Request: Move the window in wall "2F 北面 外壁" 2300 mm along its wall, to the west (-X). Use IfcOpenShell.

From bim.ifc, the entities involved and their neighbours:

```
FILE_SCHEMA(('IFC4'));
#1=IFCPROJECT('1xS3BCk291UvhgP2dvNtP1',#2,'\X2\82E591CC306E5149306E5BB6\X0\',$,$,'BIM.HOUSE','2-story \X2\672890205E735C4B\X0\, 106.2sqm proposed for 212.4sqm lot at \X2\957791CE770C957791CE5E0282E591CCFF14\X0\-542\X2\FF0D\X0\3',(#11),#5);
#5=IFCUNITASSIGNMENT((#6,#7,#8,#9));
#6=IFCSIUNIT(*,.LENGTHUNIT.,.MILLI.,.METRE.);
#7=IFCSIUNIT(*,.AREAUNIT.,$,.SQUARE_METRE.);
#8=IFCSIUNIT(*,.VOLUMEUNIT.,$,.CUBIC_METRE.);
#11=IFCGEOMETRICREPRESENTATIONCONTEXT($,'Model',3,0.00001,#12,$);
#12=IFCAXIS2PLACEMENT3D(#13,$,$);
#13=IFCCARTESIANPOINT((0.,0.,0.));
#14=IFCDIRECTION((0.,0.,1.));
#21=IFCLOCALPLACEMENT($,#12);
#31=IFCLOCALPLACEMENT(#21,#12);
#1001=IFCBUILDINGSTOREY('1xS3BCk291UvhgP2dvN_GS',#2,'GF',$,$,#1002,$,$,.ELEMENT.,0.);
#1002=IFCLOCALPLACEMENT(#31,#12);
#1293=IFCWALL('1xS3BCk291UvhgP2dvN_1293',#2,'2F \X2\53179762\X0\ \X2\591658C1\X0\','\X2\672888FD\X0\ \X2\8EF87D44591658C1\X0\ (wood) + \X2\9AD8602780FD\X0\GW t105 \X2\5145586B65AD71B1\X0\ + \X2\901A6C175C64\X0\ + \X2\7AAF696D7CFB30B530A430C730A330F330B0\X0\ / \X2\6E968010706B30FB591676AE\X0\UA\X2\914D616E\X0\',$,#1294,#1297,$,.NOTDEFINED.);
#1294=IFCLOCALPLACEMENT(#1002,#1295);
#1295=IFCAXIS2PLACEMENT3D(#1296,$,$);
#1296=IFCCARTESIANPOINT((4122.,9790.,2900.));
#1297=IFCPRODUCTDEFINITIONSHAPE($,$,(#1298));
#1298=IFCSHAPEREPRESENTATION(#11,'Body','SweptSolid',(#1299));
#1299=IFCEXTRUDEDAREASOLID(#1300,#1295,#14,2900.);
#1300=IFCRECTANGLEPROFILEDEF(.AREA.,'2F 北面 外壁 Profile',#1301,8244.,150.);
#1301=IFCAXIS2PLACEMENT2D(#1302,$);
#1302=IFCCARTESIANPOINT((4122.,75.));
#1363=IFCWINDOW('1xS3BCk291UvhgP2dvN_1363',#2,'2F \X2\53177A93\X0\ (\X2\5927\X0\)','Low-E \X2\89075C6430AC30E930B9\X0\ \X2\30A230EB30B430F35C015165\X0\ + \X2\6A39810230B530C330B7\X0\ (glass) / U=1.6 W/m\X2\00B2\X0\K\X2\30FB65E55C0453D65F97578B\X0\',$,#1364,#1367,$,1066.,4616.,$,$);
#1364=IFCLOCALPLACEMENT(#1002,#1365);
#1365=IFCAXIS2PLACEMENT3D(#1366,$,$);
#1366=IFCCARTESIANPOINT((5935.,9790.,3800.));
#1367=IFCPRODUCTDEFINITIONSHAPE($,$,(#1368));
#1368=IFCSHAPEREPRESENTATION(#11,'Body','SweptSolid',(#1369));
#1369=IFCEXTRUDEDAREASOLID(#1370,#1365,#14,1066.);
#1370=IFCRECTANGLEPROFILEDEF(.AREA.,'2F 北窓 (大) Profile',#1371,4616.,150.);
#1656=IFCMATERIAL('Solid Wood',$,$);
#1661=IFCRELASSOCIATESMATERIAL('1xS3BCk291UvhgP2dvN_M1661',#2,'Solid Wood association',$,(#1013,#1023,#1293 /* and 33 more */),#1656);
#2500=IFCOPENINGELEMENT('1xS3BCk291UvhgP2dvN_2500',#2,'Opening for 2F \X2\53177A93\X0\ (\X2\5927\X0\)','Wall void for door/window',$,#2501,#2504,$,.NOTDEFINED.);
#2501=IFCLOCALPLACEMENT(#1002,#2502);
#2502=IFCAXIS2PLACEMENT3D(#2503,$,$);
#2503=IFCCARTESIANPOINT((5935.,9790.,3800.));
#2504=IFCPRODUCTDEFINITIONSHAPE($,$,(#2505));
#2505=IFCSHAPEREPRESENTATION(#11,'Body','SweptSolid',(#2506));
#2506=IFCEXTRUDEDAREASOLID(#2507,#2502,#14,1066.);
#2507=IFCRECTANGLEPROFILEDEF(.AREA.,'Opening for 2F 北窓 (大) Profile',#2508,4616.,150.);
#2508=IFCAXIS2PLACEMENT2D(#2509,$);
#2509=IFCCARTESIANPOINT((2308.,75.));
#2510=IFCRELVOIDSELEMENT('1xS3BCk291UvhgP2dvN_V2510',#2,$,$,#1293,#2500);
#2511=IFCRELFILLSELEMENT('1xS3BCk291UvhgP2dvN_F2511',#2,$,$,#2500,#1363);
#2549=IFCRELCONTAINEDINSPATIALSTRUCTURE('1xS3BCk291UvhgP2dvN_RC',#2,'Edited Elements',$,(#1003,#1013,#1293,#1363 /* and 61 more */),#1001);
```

```python
import ifcopenshell
import ifcopenshell.api.geometry
import ifcopenshell.util.placement
import ifcopenshell.util.unit

model = ifcopenshell.open("bim.ifc")
unit_scale = ifcopenshell.util.unit.calculate_unit_scale(model)

window = model.by_guid("1xS3BCk291UvhgP2dvN_1363")
opening = window.FillsVoids[0].RelatingOpeningElement
wall = opening.VoidsElements[0].RelatingBuildingElement

wall_matrix = ifcopenshell.util.placement.get_local_placement(wall.ObjectPlacement)
shift = wall_matrix[:3, 0] * -2.3 / unit_scale
before = ifcopenshell.util.placement.get_local_placement(window.ObjectPlacement)[:3, 3].copy()

# The window is not placed relative to its opening, so move both.
for product in (opening, window):
    matrix = ifcopenshell.util.placement.get_local_placement(product.ObjectPlacement)
    matrix[:3, 3] += shift
    ifcopenshell.api.geometry.edit_object_placement(model, product=product, matrix=matrix, is_si=False)

after = ifcopenshell.util.placement.get_local_placement(window.ObjectPlacement)[:3, 3]
print("window moved by", (after - before).round(3) + 0.0)

model.write("bim_v2.ifc")
```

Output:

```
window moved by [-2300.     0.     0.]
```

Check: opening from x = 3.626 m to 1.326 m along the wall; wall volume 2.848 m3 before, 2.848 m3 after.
